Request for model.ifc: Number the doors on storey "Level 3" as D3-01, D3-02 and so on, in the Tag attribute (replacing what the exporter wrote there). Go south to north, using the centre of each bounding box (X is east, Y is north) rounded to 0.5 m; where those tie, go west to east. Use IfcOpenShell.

First a look at what the model holds.

```python
import ifcopenshell
import ifcopenshell.util.element
import ifcopenshell.util.placement

model = ifcopenshell.open("model.ifc")
print(model.schema)
storey = next(s for s in model.by_type("IfcBuildingStorey") if s.Name == "Level 3")
doors = [e for e in ifcopenshell.util.element.get_decomposition(storey) if e.is_a("IfcDoor")]
for e in sorted(doors, key=lambda e: e.id()):
    origin = ifcopenshell.util.placement.get_local_placement(e.ObjectPlacement)[:3, 3]
    print(e.id(), e.Tag, e.Name, origin.round(2) + 0.0, sep=" | ")
```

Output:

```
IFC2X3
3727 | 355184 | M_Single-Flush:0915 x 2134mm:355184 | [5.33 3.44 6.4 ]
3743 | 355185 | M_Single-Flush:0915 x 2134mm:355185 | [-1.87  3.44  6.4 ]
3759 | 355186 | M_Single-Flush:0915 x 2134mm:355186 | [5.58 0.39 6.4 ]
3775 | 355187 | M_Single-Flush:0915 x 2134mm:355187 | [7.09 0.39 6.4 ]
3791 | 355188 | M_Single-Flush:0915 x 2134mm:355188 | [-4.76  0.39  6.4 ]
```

```python
import ifcopenshell
import ifcopenshell.geom
import ifcopenshell.util.element
import ifcopenshell.util.shape

model = ifcopenshell.open("model.ifc")
settings = ifcopenshell.geom.settings()
settings.set("use-world-coords", True)


def centre(element):
    shape = ifcopenshell.geom.create_shape(settings, element)
    return ifcopenshell.util.shape.get_bbox_centroid(shape.geometry)


storey = next(s for s in model.by_type("IfcBuildingStorey") if s.Name == "Level 3")
doors = [e for e in ifcopenshell.util.element.get_decomposition(storey) if e.is_a("IfcDoor")]

# Insertion points can sit at a corner or the storey origin, so sort by the geometry (in metres).
centres = {e: centre(e) for e in doors}
doors.sort(key=lambda e: (round(centres[e][1] / 0.5), centres[e][0]))

for i, e in enumerate(doors, start=1):
    number = f"D3-{i:02d}"
    e.Tag = number
    print(e.id(), number)

model.write("model_rev.ifc")
```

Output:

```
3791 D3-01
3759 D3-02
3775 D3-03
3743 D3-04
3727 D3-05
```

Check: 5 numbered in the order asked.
